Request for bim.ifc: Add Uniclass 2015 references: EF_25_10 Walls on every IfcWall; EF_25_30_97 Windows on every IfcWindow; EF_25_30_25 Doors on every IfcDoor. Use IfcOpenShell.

First a look at what the model holds.

```python
import ifcopenshell

model = ifcopenshell.open("bim.ifc")
print(model.schema)
print("classifications:", [c.Name for c in model.by_type("IfcClassification")])
for ifc_class in ("IfcDoor", "IfcRoof", "IfcStair", "IfcWall", "IfcWindow"):
    print(ifc_class, len(model.by_type(ifc_class)))
```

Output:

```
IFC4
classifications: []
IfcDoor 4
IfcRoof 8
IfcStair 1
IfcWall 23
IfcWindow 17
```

```python
import ifcopenshell
import ifcopenshell.api.classification

model = ifcopenshell.open("bim.ifc")

system = ifcopenshell.api.classification.add_classification(model, classification="Uniclass 2015")

codes = {
    "IfcWall": ("EF_25_10", "Walls"),
    "IfcWindow": ("EF_25_30_97", "Windows"),
    "IfcDoor": ("EF_25_30_25", "Doors"),
}
for ifc_class, (code, name) in codes.items():
    products = model.by_type(ifc_class)
    ifcopenshell.api.classification.add_reference(
        model, products=products, classification=system, identification=code, name=name
    )
    print(code, len(products))

model.write("bim_edited.ifc")
```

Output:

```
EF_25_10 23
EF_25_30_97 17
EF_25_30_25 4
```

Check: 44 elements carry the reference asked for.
